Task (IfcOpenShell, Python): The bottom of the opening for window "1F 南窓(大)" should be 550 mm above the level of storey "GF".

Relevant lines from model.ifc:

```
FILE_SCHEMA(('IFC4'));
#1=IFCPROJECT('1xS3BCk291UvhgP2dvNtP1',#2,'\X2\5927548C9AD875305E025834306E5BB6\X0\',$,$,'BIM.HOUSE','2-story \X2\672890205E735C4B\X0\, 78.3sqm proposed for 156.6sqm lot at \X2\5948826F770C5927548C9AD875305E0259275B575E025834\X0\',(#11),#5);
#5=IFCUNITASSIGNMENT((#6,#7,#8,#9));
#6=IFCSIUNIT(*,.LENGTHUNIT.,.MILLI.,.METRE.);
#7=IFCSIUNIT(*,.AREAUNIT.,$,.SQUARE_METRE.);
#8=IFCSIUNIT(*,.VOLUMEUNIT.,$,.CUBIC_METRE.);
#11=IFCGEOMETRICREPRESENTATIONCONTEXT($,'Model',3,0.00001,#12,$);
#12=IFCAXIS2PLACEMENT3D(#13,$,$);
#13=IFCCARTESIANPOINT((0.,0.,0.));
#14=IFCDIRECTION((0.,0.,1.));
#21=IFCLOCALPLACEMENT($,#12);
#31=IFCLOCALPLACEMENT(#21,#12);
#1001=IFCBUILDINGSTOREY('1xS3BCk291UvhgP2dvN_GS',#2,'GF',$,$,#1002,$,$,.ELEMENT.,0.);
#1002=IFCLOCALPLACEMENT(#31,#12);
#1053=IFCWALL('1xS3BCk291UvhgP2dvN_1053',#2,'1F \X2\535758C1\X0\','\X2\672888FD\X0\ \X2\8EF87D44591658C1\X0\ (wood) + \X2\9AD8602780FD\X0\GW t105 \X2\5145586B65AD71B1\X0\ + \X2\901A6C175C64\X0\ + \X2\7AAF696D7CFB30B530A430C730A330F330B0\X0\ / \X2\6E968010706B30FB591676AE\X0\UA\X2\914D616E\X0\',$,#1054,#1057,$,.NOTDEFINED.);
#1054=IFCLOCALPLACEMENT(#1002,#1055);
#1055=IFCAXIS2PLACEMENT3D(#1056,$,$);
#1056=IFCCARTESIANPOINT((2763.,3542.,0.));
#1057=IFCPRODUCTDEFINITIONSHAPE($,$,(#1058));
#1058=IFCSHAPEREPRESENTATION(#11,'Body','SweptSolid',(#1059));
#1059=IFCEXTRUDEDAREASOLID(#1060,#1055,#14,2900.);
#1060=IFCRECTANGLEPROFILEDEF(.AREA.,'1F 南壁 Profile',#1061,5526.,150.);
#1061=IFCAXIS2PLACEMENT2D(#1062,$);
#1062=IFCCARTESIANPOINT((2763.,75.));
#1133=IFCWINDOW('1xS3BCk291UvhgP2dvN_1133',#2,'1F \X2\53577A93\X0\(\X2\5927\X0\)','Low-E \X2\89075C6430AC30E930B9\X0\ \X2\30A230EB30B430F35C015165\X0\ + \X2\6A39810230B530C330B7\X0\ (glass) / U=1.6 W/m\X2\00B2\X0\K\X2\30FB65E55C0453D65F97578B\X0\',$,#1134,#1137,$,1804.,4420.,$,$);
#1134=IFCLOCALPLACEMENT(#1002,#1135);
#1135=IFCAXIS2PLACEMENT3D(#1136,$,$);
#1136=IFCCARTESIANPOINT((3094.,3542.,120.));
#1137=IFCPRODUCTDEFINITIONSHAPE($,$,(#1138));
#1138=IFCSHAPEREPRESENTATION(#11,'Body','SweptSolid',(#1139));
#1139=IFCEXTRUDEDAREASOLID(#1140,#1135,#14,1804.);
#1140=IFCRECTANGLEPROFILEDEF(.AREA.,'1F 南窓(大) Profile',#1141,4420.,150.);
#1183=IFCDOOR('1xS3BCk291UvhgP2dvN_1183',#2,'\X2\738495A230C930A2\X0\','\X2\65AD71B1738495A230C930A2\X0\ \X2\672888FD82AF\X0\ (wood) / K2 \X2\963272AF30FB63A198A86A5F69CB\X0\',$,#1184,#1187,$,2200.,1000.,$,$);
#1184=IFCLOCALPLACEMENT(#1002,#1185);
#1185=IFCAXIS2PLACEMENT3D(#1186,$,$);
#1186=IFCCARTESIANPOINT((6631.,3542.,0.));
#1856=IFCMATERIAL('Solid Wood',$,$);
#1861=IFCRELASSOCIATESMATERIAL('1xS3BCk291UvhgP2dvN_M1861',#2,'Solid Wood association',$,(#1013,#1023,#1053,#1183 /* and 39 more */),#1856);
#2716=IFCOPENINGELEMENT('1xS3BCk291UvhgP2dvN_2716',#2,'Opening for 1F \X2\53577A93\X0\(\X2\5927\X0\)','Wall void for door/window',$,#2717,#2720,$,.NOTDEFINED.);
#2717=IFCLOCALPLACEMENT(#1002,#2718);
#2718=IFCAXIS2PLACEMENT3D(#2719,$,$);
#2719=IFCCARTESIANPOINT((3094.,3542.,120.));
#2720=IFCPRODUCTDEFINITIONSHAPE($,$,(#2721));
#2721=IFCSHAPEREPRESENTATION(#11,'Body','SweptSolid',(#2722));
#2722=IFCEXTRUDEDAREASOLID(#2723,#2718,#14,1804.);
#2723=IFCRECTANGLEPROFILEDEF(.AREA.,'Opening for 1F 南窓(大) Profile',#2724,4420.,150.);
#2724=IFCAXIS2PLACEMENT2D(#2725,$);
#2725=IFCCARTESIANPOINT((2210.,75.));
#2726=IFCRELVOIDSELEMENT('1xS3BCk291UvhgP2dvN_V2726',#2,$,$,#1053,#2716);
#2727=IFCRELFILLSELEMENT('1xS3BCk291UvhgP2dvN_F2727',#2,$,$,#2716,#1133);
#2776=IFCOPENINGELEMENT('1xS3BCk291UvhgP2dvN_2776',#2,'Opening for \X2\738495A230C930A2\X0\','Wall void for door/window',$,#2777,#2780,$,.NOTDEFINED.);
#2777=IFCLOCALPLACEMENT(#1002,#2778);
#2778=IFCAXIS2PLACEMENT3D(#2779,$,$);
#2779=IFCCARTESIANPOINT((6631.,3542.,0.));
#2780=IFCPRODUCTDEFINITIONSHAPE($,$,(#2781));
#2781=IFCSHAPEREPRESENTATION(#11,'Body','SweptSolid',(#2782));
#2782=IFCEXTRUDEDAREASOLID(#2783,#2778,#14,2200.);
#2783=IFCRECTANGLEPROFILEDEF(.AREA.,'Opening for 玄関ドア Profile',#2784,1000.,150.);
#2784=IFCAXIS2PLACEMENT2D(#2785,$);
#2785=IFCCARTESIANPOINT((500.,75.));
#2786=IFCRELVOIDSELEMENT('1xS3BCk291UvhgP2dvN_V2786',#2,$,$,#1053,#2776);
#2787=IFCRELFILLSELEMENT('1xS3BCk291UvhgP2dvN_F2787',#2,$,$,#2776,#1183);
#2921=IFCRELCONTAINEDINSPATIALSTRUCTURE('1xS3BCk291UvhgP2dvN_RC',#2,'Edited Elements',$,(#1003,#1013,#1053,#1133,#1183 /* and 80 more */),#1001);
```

```python
import numpy as np
import ifcopenshell
import ifcopenshell.api.geometry
import ifcopenshell.geom
import ifcopenshell.util.element
import ifcopenshell.util.placement
import ifcopenshell.util.shape
import ifcopenshell.util.unit

model = ifcopenshell.open("model.ifc")
unit_scale = ifcopenshell.util.unit.calculate_unit_scale(model)

window = model.by_id(1133)
opening = window.FillsVoids[0].RelatingOpeningElement
storey = ifcopenshell.util.element.get_container(window, ifc_class="IfcBuildingStorey")
level = ifcopenshell.util.placement.get_local_placement(storey.ObjectPlacement)[2, 3]

# The opening's origin need not be at the sill, so measure its lowest point.
shape = ifcopenshell.geom.create_shape(ifcopenshell.geom.settings(), opening)
bottom = ifcopenshell.util.shape.get_shape_bottom_elevation(shape, shape.geometry) / unit_scale
dz = level + 0.55 / unit_scale - bottom

shift = np.array([0.0, 0.0, dz])
# The window is not placed relative to its opening, so move both.
for product in (opening, window):
    matrix = ifcopenshell.util.placement.get_local_placement(product.ObjectPlacement)
    matrix[:3, 3] += shift
    ifcopenshell.api.geometry.edit_object_placement(model, product=product, matrix=matrix, is_si=False)

print(f"moved by {dz * unit_scale:+.3f} m")

model.write("model_updated.ifc")
```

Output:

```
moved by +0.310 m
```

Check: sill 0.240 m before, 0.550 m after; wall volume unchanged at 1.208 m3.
